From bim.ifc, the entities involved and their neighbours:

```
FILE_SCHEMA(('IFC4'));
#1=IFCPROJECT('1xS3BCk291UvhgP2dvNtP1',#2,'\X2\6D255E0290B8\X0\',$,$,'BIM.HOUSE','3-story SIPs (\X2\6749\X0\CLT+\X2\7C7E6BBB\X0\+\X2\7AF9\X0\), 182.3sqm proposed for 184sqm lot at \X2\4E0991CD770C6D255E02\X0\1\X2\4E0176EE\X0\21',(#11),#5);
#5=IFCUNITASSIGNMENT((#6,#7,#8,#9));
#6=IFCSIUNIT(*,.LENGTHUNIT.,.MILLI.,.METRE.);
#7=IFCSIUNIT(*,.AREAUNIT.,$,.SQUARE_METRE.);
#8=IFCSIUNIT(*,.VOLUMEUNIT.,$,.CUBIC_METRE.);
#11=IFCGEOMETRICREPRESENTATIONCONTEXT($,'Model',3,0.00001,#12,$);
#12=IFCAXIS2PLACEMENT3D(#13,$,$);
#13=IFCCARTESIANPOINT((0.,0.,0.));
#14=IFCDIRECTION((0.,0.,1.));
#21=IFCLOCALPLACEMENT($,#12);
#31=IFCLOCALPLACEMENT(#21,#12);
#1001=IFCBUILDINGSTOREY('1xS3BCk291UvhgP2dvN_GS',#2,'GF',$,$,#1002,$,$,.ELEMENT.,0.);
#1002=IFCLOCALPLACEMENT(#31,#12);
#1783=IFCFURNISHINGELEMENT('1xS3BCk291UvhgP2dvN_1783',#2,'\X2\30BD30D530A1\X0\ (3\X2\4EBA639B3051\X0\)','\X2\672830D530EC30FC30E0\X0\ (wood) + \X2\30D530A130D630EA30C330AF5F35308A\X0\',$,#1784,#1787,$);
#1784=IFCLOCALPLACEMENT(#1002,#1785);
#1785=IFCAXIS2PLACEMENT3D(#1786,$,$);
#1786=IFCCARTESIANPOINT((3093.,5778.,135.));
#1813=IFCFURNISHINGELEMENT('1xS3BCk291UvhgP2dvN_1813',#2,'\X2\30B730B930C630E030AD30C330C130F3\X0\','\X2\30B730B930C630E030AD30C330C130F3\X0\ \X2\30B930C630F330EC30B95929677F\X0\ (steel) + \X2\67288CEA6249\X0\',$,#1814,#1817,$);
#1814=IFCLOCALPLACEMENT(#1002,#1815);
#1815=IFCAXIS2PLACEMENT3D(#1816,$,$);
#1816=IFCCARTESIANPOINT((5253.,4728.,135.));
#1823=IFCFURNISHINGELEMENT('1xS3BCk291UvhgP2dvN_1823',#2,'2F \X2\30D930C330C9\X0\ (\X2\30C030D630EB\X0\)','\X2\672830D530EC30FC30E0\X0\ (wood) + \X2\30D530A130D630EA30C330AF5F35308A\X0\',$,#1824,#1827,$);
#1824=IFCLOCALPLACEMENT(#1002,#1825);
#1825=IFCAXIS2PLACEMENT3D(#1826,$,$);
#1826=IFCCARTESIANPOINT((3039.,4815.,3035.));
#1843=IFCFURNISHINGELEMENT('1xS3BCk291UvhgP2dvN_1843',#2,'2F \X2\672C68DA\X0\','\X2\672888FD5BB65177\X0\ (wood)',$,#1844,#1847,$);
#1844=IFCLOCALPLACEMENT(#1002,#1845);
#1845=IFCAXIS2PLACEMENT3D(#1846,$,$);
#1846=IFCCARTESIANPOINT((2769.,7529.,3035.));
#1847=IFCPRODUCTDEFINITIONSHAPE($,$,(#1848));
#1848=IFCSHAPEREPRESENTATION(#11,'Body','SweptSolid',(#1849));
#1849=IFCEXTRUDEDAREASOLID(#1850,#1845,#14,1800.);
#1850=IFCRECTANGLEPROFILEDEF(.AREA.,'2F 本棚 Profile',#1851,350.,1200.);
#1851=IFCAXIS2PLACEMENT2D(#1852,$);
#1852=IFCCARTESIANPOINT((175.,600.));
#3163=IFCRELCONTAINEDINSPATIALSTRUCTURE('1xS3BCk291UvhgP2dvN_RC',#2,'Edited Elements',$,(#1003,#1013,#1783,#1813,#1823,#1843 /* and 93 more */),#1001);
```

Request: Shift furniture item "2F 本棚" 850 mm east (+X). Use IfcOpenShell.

```python
import ifcopenshell
import ifcopenshell.api.geometry
import ifcopenshell.util.placement

model = ifcopenshell.open("bim.ifc")

item = model.by_id(1843)
matrix = ifcopenshell.util.placement.get_local_placement(item.ObjectPlacement)
matrix[0, 3] += 850.0
ifcopenshell.api.geometry.edit_object_placement(model, product=item, matrix=matrix, is_si=False)

print(ifcopenshell.util.placement.get_local_placement(item.ObjectPlacement).round(3) + 0.0)

model.write("bim-out.ifc")
```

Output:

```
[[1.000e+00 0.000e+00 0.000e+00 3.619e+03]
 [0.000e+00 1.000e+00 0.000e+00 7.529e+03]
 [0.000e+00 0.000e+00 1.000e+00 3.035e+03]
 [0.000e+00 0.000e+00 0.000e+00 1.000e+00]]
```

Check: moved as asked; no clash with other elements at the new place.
